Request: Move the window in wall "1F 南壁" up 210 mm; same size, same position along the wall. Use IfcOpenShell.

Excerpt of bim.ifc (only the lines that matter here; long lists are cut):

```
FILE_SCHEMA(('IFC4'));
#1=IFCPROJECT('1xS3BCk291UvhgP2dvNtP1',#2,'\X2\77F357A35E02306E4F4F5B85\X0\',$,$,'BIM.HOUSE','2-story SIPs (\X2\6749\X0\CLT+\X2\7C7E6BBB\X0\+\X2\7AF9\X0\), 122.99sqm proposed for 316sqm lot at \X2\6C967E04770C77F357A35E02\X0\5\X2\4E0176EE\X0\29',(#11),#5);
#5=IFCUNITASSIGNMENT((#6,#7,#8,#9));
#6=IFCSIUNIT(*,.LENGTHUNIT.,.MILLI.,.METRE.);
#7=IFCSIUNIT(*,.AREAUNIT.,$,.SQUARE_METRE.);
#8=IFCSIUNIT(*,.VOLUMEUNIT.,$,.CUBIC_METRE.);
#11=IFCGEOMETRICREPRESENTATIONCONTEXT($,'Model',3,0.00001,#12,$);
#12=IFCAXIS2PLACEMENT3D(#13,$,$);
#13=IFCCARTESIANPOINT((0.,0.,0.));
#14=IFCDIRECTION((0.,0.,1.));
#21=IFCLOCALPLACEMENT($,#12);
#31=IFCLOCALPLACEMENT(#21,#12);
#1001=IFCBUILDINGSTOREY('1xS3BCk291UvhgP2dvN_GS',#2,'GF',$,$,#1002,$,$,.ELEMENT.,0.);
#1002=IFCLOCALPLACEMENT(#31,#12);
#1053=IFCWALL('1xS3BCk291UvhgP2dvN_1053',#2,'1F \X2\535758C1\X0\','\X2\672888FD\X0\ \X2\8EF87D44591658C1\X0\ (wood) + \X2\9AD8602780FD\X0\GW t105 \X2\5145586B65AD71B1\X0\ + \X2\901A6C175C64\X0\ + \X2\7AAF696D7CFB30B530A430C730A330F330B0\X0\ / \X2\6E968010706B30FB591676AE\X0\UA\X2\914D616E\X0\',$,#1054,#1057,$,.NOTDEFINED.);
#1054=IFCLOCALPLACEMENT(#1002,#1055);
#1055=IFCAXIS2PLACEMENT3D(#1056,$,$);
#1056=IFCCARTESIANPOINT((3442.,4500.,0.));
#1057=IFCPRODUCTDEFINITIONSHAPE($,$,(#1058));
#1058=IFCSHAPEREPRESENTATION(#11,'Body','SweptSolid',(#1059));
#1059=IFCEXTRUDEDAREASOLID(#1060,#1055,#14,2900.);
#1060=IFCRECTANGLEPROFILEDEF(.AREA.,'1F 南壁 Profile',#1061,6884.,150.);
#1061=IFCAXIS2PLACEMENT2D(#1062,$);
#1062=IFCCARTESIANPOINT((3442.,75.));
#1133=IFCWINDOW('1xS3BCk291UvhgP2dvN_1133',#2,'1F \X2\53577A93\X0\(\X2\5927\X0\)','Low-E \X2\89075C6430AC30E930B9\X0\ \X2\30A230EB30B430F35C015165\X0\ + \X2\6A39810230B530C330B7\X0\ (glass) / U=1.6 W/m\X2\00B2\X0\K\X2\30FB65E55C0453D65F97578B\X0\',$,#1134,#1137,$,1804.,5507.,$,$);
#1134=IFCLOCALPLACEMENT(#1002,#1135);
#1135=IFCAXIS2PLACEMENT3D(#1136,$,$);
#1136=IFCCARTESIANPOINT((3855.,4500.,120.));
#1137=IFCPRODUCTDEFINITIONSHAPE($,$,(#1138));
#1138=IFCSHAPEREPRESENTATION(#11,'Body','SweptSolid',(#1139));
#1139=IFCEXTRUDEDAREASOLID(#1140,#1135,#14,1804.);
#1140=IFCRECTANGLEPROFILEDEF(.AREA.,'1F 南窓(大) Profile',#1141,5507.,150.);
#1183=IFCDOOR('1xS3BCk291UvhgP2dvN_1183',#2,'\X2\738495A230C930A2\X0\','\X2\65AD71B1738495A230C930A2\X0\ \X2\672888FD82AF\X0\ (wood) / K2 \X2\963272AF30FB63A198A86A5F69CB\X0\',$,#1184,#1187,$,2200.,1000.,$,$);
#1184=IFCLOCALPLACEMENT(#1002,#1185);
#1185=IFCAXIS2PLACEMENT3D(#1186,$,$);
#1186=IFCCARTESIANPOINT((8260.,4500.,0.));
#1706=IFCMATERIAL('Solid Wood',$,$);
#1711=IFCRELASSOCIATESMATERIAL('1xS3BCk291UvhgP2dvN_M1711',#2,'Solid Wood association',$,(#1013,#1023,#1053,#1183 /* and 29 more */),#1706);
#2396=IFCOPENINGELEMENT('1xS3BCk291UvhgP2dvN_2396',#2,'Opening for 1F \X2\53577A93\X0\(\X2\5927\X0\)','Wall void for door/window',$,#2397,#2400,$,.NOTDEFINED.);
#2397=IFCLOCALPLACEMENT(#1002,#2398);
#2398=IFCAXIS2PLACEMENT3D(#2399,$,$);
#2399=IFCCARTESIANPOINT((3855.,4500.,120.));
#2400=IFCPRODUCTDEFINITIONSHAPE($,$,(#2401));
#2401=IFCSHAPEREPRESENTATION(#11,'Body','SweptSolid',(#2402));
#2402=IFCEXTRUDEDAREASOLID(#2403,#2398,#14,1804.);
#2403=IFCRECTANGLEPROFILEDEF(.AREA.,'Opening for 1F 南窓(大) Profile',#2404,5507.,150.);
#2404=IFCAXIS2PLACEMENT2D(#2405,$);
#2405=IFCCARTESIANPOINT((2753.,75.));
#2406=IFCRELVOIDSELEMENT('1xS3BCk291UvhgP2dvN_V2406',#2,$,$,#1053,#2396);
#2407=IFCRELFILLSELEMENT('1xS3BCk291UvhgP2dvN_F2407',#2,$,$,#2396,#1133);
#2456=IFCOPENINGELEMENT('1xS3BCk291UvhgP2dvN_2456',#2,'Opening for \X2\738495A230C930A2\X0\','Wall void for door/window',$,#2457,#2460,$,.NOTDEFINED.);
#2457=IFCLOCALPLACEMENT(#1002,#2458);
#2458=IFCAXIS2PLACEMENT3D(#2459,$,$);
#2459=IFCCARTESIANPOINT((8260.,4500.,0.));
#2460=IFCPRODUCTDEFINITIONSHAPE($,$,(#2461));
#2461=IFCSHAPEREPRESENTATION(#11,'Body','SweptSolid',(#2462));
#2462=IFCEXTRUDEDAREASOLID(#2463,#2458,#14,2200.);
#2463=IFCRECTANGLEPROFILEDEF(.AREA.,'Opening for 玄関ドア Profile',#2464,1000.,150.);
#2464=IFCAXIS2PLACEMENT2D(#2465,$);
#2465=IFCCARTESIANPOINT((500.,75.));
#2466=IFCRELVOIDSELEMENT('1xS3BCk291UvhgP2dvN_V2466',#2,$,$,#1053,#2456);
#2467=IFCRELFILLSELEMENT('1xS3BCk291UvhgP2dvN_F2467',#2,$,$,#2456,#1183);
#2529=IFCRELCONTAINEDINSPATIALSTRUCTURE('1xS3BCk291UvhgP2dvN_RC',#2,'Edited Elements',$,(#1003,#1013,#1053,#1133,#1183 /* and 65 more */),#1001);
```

```python
import numpy as np
import ifcopenshell
import ifcopenshell.api.geometry
import ifcopenshell.util.placement
import ifcopenshell.util.unit

model = ifcopenshell.open("bim.ifc")
unit_scale = ifcopenshell.util.unit.calculate_unit_scale(model)

window = model.by_guid("1xS3BCk291UvhgP2dvN_1133")
opening = window.FillsVoids[0].RelatingOpeningElement
dz = 210.0

shift = np.array([0.0, 0.0, dz])
# The window is not placed relative to its opening, so move both.
for product in (opening, window):
    matrix = ifcopenshell.util.placement.get_local_placement(product.ObjectPlacement)
    matrix[:3, 3] += shift
    ifcopenshell.api.geometry.edit_object_placement(model, product=product, matrix=matrix, is_si=False)

print(f"moved by {dz * unit_scale:+.3f} m")

model.write("bim_v2.ifc")
```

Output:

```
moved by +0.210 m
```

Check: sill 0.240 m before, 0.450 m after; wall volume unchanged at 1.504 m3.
